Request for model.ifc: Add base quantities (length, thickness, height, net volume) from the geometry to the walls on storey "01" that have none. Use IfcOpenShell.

First a look at what the model holds.

```python
import ifcopenshell
import ifcopenshell.util.element
import ifcopenshell.util.unit

model = ifcopenshell.open("model.ifc")
print(model.schema)
for unit_type in ("LENGTHUNIT", "AREAUNIT", "VOLUMEUNIT"):
    print(unit_type, ifcopenshell.util.unit.calculate_unit_scale(model, unit_type))
storey = next(s for s in model.by_type("IfcBuildingStorey") if s.Name == "01")
walls = [e for e in ifcopenshell.util.element.get_decomposition(storey) if e.is_a("IfcWall")]
for e in sorted(walls, key=lambda e: e.id()):
    print(e.id(), e.is_a(), e.Name, list(ifcopenshell.util.element.get_psets(e, qtos_only=True)), sep=" | ")
```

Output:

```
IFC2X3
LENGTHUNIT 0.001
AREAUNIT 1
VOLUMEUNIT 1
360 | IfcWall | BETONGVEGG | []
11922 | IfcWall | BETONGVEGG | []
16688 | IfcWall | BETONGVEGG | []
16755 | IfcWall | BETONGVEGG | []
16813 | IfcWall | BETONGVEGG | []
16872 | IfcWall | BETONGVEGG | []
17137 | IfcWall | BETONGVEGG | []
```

```python
import ifcopenshell
import ifcopenshell.api.pset
import ifcopenshell.geom
import ifcopenshell.util.element
import ifcopenshell.util.shape
import ifcopenshell.util.unit

model = ifcopenshell.open("model.ifc")
unit_scale = ifcopenshell.util.unit.calculate_unit_scale(model)
volume_scale = ifcopenshell.util.unit.calculate_unit_scale(model, "VOLUMEUNIT")
settings = ifcopenshell.geom.settings()

storey = next(s for s in model.by_type("IfcBuildingStorey") if s.Name == "01")
walls = [e for e in ifcopenshell.util.element.get_decomposition(storey) if e.is_a("IfcWall")]

for e in sorted(walls, key=lambda e: e.id()):
    if ifcopenshell.util.element.get_psets(e, qtos_only=True, should_inherit=False):
        continue
    # Geometry comes back in metres, in the element's own axes.
    shape = ifcopenshell.geom.create_shape(settings, e)
    values = {
        "Length": ifcopenshell.util.shape.get_x(shape.geometry) / unit_scale,
        "Width": ifcopenshell.util.shape.get_y(shape.geometry) / unit_scale,
        "Height": ifcopenshell.util.shape.get_z(shape.geometry) / unit_scale,
        "NetVolume": ifcopenshell.util.shape.get_volume(shape.geometry) / volume_scale,
    }
    qto = ifcopenshell.api.pset.add_qto(model, product=e, name="BaseQuantities")
    ifcopenshell.api.pset.edit_qto(model, qto=qto, properties=values)
    print(e.id(), {k: round(v, 3) for k, v in values.items()})

model.write("model_rev.ifc")
```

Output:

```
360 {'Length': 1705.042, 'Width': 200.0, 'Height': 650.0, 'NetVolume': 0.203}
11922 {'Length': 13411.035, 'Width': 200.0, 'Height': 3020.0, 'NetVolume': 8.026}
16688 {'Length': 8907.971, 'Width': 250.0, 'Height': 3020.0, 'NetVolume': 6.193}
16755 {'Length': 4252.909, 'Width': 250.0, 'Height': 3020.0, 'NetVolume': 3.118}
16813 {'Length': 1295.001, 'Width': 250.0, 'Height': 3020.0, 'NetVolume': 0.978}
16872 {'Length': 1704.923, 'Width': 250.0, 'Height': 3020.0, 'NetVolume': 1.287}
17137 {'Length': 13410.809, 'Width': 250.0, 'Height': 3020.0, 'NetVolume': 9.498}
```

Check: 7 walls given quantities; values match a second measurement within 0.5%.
